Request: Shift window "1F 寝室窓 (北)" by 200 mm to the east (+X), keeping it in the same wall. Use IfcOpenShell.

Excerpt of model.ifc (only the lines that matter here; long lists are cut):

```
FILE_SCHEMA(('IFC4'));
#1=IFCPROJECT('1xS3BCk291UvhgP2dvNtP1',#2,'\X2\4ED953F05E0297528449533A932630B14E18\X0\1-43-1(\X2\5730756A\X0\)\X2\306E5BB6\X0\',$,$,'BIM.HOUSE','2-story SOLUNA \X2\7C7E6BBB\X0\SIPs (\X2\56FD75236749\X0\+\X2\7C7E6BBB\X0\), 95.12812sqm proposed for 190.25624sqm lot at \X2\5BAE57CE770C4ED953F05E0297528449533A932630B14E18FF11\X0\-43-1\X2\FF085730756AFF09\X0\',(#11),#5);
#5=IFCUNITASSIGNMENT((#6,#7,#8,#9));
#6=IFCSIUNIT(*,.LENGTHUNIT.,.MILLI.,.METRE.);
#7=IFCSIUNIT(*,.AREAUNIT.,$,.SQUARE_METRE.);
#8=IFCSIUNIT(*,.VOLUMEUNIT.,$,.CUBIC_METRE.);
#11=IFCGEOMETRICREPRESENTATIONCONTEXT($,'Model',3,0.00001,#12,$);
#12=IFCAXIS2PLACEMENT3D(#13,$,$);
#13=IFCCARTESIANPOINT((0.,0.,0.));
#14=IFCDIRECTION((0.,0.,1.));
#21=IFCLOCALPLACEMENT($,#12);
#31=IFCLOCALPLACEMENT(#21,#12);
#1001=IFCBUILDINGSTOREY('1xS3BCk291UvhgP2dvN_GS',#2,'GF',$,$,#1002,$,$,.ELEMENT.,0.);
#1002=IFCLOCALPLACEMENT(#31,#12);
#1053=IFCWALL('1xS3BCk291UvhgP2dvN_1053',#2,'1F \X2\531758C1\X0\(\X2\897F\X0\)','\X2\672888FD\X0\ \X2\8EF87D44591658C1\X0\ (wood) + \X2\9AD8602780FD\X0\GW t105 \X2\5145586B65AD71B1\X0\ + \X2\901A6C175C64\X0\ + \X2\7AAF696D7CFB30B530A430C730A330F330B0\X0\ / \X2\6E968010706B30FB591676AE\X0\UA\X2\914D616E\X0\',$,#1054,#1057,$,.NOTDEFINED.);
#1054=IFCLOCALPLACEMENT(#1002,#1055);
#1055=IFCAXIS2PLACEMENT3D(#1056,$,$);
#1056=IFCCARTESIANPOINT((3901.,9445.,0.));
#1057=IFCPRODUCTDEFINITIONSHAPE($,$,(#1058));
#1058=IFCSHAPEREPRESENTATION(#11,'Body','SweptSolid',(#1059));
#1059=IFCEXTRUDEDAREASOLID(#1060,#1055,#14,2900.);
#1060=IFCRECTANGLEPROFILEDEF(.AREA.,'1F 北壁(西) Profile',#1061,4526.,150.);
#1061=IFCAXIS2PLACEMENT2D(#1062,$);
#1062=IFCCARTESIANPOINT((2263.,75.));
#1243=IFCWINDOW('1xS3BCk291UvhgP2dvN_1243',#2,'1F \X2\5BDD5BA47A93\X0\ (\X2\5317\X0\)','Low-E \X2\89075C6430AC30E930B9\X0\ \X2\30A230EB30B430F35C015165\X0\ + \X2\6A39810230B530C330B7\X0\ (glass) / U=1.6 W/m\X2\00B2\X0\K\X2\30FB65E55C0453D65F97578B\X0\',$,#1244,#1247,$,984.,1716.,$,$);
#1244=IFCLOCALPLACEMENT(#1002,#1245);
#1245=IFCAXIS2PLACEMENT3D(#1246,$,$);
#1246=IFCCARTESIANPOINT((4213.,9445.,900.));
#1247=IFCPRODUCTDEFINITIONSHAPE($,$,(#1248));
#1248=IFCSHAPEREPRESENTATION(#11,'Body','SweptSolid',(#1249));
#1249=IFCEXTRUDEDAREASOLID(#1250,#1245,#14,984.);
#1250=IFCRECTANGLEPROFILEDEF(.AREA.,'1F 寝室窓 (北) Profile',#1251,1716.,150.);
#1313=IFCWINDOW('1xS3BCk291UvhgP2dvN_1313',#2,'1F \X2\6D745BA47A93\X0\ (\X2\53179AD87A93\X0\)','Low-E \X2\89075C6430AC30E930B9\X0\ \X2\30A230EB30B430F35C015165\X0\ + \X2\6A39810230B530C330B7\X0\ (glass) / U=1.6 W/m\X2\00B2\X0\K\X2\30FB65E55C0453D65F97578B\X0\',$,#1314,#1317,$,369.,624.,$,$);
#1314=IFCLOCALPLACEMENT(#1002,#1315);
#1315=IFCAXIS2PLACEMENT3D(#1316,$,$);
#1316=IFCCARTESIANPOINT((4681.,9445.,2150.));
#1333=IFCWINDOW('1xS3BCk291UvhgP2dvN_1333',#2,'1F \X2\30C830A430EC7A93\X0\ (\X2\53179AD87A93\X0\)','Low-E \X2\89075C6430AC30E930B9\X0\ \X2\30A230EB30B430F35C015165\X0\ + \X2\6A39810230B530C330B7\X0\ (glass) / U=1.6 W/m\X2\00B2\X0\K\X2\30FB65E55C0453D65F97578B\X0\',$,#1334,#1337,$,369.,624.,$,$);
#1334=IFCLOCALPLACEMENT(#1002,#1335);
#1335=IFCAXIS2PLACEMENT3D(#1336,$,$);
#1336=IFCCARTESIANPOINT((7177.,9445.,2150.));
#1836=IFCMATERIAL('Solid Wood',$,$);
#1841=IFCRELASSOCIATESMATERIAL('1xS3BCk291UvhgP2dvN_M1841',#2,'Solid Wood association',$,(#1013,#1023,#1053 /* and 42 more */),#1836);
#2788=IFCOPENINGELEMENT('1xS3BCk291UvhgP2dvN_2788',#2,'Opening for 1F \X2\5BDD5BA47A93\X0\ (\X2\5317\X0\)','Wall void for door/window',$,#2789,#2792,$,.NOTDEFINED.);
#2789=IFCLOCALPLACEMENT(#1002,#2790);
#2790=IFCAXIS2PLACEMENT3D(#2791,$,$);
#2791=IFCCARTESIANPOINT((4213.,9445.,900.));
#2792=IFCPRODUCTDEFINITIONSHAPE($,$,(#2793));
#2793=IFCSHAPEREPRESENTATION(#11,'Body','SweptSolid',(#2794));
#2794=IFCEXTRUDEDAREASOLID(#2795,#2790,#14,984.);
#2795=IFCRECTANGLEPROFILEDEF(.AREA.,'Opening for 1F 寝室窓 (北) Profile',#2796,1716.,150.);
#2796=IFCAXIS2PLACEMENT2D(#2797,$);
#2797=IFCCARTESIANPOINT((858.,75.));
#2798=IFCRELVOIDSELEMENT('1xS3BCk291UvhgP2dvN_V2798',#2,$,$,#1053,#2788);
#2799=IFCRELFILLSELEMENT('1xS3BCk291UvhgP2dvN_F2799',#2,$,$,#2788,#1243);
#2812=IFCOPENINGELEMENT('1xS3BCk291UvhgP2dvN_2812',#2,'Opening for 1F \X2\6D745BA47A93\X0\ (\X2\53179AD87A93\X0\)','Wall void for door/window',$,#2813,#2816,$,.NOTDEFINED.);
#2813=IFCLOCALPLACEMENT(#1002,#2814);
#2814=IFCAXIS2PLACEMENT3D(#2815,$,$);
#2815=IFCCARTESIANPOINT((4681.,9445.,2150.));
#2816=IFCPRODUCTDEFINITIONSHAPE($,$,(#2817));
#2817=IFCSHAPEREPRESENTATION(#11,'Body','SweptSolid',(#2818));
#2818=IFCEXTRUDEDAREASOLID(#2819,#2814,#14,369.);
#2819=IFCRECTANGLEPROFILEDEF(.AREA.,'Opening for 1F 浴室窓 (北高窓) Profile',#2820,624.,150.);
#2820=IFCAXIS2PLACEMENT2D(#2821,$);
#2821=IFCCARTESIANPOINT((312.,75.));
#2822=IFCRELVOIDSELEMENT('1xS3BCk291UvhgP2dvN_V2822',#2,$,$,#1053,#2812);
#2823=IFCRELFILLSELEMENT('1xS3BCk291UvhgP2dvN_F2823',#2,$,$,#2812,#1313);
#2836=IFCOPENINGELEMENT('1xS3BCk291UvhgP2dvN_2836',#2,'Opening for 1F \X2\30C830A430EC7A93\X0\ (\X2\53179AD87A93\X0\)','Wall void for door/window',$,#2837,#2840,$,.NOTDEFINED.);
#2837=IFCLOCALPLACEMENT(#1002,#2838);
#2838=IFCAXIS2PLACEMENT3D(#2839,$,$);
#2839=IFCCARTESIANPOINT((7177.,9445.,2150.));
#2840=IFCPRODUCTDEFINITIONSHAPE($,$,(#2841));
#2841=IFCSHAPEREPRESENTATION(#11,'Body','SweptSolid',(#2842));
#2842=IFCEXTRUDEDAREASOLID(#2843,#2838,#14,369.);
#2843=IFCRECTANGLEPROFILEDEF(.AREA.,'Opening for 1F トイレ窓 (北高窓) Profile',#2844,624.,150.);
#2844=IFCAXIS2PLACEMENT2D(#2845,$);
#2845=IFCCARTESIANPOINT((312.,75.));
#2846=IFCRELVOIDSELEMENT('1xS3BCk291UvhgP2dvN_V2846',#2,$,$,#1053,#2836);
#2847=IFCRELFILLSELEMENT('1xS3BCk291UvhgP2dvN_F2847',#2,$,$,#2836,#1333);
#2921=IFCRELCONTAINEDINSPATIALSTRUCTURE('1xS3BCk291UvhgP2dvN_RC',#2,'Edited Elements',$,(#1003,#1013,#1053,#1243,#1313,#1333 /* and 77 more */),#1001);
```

```python
import ifcopenshell
import ifcopenshell.api.geometry
import ifcopenshell.util.placement
import ifcopenshell.util.unit

model = ifcopenshell.open("model.ifc")
unit_scale = ifcopenshell.util.unit.calculate_unit_scale(model)

window = model.by_id(1243)
opening = window.FillsVoids[0].RelatingOpeningElement
wall = opening.VoidsElements[0].RelatingBuildingElement

wall_matrix = ifcopenshell.util.placement.get_local_placement(wall.ObjectPlacement)
shift = wall_matrix[:3, 0] * 0.2 / unit_scale
before = ifcopenshell.util.placement.get_local_placement(window.ObjectPlacement)[:3, 3].copy()

# The window is not placed relative to its opening, so move both.
for product in (opening, window):
    matrix = ifcopenshell.util.placement.get_local_placement(product.ObjectPlacement)
    matrix[:3, 3] += shift
    ifcopenshell.api.geometry.edit_object_placement(model, product=product, matrix=matrix, is_si=False)

after = ifcopenshell.util.placement.get_local_placement(window.ObjectPlacement)[:3, 3]
print("window moved by", (after - before).round(3) + 0.0)

model.write("model_rev.ifc")
```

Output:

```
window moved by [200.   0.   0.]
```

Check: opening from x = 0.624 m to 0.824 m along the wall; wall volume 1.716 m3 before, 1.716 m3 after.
